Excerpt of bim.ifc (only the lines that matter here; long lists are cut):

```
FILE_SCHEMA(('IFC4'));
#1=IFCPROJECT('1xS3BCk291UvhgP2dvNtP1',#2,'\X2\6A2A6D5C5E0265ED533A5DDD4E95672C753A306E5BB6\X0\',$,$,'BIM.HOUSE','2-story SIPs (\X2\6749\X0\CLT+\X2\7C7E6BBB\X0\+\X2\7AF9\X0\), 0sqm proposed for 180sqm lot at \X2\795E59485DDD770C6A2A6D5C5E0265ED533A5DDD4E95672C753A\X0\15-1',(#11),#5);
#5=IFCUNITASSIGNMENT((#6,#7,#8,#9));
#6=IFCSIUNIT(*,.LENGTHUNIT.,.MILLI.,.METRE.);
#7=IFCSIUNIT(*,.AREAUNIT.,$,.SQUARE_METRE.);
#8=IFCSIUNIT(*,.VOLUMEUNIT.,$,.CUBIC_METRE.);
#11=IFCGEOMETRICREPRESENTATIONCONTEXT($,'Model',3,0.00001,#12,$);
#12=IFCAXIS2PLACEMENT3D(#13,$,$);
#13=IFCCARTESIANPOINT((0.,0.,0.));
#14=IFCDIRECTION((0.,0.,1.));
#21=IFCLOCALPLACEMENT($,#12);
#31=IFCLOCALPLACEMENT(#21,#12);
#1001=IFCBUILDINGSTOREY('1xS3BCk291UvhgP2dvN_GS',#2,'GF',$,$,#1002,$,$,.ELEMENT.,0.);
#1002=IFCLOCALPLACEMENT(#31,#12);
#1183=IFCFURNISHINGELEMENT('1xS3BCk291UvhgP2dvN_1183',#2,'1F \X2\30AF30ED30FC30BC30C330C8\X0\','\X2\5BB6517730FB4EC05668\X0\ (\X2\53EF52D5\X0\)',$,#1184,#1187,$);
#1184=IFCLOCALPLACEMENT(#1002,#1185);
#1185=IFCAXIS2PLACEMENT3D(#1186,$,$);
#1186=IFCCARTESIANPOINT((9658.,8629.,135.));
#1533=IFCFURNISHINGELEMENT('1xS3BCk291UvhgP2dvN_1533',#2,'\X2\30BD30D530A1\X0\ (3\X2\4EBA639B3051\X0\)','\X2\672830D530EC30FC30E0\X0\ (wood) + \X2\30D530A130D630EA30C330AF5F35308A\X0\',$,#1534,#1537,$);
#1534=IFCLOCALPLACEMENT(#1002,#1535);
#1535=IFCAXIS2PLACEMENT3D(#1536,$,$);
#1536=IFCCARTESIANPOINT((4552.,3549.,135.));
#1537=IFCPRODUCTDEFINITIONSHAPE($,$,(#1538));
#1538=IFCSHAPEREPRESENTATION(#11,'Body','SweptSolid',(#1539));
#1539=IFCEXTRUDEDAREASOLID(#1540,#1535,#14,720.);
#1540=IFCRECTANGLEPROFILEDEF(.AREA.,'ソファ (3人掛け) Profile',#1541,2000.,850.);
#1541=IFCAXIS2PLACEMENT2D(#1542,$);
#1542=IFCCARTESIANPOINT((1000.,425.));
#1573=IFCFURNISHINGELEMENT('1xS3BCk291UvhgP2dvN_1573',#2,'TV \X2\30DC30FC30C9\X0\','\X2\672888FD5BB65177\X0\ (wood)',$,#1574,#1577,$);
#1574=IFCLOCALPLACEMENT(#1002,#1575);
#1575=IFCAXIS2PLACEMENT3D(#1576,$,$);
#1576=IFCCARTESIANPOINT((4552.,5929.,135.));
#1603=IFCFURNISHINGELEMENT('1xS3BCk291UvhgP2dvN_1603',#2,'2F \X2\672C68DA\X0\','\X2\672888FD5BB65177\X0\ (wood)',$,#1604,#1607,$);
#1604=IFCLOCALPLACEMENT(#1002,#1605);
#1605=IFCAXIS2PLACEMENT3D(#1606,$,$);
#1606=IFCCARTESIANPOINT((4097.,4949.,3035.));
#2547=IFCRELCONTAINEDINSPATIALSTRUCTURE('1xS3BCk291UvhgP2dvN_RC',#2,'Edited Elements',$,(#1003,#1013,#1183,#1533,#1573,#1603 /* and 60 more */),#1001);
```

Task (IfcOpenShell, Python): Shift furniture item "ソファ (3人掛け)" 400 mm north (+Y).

```python
import ifcopenshell
import ifcopenshell.api.geometry
import ifcopenshell.util.placement
import ifcopenshell.util.unit

model = ifcopenshell.open("bim.ifc")
unit_scale = ifcopenshell.util.unit.calculate_unit_scale(model)

item = model.by_guid("1xS3BCk291UvhgP2dvN_1533")
matrix = ifcopenshell.util.placement.get_local_placement(item.ObjectPlacement)
matrix[1, 3] += 0.4 / unit_scale
ifcopenshell.api.geometry.edit_object_placement(model, product=item, matrix=matrix, is_si=False)

print(ifcopenshell.util.placement.get_local_placement(item.ObjectPlacement).round(3) + 0.0)

model.write("bim_updated.ifc")
```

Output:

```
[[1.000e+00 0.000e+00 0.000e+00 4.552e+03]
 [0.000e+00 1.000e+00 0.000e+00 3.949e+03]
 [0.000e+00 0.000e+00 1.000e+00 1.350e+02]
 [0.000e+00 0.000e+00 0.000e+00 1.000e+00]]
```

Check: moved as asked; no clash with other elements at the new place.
